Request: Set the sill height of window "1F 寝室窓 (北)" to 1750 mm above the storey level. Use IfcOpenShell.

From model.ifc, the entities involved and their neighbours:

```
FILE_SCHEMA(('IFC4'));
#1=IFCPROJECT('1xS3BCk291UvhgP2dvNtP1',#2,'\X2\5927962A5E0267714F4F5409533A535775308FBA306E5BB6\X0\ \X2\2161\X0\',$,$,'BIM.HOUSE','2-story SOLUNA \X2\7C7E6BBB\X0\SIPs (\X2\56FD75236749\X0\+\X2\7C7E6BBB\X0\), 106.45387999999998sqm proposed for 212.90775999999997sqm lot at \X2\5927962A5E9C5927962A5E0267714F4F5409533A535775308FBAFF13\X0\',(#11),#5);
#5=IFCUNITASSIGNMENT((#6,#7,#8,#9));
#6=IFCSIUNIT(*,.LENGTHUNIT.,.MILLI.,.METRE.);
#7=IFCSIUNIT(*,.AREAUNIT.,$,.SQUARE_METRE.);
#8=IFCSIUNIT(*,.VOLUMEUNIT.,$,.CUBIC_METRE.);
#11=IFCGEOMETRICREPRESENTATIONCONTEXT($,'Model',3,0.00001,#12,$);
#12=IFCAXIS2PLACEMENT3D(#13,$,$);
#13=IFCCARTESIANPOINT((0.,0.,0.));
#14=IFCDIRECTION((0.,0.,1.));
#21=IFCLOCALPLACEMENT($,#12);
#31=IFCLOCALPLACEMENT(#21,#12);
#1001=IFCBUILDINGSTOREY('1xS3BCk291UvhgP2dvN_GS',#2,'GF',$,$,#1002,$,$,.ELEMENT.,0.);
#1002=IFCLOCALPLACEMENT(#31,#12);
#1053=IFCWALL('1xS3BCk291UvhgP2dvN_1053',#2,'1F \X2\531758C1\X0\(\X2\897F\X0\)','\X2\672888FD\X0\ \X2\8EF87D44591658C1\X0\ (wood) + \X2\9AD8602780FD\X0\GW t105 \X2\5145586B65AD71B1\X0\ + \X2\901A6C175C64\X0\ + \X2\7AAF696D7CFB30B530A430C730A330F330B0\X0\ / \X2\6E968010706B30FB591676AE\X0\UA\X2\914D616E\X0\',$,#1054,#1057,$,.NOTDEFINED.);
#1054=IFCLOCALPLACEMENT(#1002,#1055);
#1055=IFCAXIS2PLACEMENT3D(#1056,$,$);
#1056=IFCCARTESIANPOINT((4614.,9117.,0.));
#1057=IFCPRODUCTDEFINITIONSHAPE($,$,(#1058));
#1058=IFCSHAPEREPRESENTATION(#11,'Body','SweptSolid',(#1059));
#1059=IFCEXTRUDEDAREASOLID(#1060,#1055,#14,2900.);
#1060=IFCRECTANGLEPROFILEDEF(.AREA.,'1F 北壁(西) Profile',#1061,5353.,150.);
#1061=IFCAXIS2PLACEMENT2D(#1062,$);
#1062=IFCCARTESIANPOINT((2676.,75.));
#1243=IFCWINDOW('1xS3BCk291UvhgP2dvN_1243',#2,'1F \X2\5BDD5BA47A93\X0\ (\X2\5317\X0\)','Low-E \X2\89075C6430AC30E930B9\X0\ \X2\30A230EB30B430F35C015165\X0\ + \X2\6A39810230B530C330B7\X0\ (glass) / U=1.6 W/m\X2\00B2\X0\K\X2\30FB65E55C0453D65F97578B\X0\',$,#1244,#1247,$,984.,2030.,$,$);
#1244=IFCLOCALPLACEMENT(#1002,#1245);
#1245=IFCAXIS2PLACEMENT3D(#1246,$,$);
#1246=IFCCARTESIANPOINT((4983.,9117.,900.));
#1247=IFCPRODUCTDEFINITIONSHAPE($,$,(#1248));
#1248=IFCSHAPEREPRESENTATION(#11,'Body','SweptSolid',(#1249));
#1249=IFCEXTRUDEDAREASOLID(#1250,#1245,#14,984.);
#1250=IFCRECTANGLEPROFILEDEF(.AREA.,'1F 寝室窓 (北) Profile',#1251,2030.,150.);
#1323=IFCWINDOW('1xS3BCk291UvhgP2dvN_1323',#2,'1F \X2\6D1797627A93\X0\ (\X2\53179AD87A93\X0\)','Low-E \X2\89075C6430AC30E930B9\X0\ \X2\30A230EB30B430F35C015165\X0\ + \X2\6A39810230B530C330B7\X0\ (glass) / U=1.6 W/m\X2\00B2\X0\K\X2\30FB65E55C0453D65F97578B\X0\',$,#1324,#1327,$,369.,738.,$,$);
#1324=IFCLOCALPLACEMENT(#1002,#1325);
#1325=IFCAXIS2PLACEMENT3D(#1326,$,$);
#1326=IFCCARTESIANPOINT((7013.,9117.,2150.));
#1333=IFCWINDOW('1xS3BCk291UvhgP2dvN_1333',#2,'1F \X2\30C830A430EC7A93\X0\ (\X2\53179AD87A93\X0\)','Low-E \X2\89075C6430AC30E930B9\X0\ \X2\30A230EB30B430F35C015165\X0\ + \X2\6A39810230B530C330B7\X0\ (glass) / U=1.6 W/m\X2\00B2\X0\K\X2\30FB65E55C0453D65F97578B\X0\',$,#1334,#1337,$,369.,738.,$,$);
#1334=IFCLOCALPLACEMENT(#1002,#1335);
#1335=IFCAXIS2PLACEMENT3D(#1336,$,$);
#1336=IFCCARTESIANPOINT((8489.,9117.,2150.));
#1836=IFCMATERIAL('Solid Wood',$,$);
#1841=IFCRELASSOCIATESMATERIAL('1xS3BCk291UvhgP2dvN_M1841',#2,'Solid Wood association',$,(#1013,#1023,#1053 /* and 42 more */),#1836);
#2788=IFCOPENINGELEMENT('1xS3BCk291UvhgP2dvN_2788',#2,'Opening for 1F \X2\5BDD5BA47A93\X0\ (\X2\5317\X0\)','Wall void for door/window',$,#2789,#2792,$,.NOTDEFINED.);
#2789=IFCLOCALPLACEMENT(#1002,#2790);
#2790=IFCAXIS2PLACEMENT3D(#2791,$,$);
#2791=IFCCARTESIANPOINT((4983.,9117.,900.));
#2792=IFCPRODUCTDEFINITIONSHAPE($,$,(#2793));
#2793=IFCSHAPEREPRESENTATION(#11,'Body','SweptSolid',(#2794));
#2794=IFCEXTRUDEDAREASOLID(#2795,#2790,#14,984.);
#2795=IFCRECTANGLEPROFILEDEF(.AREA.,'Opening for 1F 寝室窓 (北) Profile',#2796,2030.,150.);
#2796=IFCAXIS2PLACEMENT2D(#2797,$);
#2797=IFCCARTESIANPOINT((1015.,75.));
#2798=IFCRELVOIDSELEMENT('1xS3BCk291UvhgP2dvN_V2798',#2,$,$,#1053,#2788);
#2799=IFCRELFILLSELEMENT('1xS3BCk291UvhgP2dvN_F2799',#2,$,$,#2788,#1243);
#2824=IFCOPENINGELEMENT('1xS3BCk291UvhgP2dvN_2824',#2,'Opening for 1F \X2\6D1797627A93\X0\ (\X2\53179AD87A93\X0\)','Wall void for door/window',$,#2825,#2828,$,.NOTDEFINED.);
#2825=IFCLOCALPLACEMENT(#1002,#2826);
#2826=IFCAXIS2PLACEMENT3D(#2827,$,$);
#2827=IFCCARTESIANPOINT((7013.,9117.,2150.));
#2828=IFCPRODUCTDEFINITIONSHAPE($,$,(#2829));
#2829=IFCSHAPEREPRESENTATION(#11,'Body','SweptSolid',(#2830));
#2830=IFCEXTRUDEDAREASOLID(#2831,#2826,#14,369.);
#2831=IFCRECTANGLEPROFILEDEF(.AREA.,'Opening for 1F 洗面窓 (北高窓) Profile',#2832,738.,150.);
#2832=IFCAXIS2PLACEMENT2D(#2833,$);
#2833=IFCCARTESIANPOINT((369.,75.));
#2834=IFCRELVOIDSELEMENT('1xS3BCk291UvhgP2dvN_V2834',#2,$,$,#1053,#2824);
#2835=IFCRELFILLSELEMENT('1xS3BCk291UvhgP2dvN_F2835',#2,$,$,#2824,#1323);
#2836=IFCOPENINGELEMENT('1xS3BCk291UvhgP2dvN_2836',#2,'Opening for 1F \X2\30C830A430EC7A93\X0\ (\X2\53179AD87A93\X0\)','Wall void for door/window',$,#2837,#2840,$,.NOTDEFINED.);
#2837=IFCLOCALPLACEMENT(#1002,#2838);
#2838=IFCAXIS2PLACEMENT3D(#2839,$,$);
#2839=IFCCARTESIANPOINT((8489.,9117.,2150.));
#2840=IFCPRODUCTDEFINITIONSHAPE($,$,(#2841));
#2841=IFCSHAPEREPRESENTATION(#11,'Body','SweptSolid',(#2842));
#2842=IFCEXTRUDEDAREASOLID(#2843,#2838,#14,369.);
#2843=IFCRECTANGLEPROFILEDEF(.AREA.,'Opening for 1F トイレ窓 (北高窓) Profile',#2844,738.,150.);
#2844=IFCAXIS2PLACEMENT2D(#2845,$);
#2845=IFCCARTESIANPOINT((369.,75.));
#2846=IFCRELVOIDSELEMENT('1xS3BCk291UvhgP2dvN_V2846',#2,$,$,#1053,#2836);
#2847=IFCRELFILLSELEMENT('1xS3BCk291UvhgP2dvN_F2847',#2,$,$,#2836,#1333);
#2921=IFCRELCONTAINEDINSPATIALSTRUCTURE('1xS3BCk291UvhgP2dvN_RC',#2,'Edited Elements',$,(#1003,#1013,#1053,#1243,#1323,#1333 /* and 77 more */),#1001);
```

```python
import numpy as np
import ifcopenshell
import ifcopenshell.api.geometry
import ifcopenshell.geom
import ifcopenshell.util.element
import ifcopenshell.util.placement
import ifcopenshell.util.shape
import ifcopenshell.util.unit

model = ifcopenshell.open("model.ifc")
unit_scale = ifcopenshell.util.unit.calculate_unit_scale(model)

window = model.by_guid("1xS3BCk291UvhgP2dvN_1243")
opening = window.FillsVoids[0].RelatingOpeningElement
storey = ifcopenshell.util.element.get_container(window, ifc_class="IfcBuildingStorey")
level = ifcopenshell.util.placement.get_local_placement(storey.ObjectPlacement)[2, 3]

# The opening's origin need not be at the sill, so measure its lowest point.
shape = ifcopenshell.geom.create_shape(ifcopenshell.geom.settings(), opening)
bottom = ifcopenshell.util.shape.get_shape_bottom_elevation(shape, shape.geometry) / unit_scale
dz = level + 1750.0 - bottom

shift = np.array([0.0, 0.0, dz])
# The window is not placed relative to its opening, so move both.
for product in (opening, window):
    matrix = ifcopenshell.util.placement.get_local_placement(product.ObjectPlacement)
    matrix[:3, 3] += shift
    ifcopenshell.api.geometry.edit_object_placement(model, product=product, matrix=matrix, is_si=False)

print(f"moved by {dz * unit_scale:+.3f} m")

model.write("model_rev.ifc")
```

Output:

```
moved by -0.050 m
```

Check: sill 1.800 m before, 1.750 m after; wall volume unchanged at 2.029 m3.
